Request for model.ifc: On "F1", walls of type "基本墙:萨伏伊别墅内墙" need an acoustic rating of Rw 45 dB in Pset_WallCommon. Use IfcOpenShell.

First a look at what the model holds.

```python
import ifcopenshell
import ifcopenshell.util.element

model = ifcopenshell.open("model.ifc")
print(model.schema)
storey = next(s for s in model.by_type("IfcBuildingStorey") if s.Name == "F1")
walls = [e for e in ifcopenshell.util.element.get_decomposition(storey) if e.is_a("IfcWall")]
seen = {}
for e in walls:
    element_type = ifcopenshell.util.element.get_type(e)
    key = (element_type.Name if element_type != e and element_type else None, ifcopenshell.util.element.get_pset(e, "Pset_WallCommon", "AcousticRating"))
    seen[key] = seen.get(key, 0) + 1
for (name, value), count in sorted(seen.items(), key=str):
    print(count, "x", name, "|", value)
```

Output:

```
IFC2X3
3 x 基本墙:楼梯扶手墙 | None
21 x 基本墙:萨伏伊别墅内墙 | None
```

```python
import ifcopenshell
import ifcopenshell.api.pset
import ifcopenshell.util.element

model = ifcopenshell.open("model.ifc")

storey = next(s for s in model.by_type("IfcBuildingStorey") if s.Name == "F1")
walls = [e for e in ifcopenshell.util.element.get_decomposition(storey) if e.is_a("IfcWall")]

count = 0
for e in walls:
    element_type = ifcopenshell.util.element.get_type(e)
    if element_type in (None, e) or element_type.Name != "基本墙:萨伏伊别墅内墙":
        continue
    # add_pset returns the element's existing set when there is one.
    pset = ifcopenshell.api.pset.add_pset(model, product=e, name="Pset_WallCommon")
    ifcopenshell.api.pset.edit_pset(model, pset=pset, properties={"AcousticRating": "Rw 45 dB"})
    count += 1

print(count, "walls updated")

model.write("model-out.ifc")
```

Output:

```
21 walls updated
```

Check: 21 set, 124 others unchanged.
